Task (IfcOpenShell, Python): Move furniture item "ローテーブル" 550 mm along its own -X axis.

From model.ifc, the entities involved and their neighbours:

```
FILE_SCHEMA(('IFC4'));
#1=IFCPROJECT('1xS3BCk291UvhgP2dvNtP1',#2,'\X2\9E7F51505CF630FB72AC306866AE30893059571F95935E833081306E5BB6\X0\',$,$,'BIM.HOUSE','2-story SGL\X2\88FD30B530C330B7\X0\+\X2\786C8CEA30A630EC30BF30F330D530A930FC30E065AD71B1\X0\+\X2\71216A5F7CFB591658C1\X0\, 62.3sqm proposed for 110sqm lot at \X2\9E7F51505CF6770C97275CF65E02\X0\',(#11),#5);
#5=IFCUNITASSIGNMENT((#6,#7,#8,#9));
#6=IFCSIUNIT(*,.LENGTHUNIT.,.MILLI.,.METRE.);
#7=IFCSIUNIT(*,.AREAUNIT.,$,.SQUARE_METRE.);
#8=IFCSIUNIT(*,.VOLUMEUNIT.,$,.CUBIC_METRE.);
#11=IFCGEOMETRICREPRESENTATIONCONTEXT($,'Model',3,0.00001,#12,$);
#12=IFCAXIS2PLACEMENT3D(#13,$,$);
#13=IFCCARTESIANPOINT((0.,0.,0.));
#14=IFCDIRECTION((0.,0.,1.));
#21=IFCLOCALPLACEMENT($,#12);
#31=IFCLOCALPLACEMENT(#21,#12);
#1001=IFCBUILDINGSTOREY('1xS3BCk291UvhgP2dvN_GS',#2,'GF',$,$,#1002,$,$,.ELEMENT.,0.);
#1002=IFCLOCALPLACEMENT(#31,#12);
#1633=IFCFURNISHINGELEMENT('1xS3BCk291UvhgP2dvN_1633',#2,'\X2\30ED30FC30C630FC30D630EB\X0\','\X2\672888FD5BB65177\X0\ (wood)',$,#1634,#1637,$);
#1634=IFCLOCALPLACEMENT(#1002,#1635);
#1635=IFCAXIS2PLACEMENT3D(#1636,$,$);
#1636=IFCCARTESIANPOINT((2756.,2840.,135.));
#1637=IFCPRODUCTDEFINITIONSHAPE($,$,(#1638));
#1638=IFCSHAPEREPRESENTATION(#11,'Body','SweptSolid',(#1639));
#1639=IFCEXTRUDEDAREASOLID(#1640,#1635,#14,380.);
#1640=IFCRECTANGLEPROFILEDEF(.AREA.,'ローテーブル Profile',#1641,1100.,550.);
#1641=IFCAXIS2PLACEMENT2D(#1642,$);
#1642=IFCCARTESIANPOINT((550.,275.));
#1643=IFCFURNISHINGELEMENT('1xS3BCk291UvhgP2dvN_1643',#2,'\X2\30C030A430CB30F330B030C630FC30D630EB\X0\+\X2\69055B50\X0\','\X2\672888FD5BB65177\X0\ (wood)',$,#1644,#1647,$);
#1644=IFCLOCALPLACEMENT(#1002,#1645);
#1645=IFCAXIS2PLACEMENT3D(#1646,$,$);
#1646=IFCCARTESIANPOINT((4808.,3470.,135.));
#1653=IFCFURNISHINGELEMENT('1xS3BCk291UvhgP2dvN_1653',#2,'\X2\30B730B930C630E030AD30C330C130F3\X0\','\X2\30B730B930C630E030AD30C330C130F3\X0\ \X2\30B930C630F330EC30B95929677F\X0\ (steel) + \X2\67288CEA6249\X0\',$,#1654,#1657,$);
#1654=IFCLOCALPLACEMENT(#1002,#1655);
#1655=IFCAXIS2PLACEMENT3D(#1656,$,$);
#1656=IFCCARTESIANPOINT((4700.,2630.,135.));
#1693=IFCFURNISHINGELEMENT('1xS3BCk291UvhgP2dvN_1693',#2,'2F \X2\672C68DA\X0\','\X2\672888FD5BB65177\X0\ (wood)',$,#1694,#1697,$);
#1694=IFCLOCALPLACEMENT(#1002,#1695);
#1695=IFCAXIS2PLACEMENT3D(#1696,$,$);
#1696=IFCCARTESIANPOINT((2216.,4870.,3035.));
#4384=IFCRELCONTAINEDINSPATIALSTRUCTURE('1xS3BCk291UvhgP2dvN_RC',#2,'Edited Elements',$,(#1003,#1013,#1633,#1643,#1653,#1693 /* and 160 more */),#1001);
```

```python
import ifcopenshell
import ifcopenshell.api.geometry
import ifcopenshell.util.placement
import ifcopenshell.util.unit

model = ifcopenshell.open("model.ifc")
unit_scale = ifcopenshell.util.unit.calculate_unit_scale(model)

item = model.by_guid("1xS3BCk291UvhgP2dvN_1633")
matrix = ifcopenshell.util.placement.get_local_placement(item.ObjectPlacement)
matrix[:3, 3] -= matrix[:3, 0] * 0.55 / unit_scale
ifcopenshell.api.geometry.edit_object_placement(model, product=item, matrix=matrix, is_si=False)

print(ifcopenshell.util.placement.get_local_placement(item.ObjectPlacement).round(3) + 0.0)

model.write("model-out.ifc")
```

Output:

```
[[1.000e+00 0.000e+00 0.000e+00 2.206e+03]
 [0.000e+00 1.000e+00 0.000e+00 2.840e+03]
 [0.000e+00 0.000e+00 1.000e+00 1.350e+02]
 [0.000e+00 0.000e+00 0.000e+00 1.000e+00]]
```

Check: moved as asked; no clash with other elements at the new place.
